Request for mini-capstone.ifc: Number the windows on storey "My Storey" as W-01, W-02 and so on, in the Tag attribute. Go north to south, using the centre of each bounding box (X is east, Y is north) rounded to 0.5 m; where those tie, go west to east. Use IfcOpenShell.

First a look at what the model holds.

```python
import ifcopenshell
import ifcopenshell.util.element
import ifcopenshell.util.placement

model = ifcopenshell.open("mini-capstone.ifc")
print(model.schema)
storey = next(s for s in model.by_type("IfcBuildingStorey") if s.Name == "My Storey")
windows = [e for e in ifcopenshell.util.element.get_decomposition(storey) if e.is_a("IfcWindow")]
for e in sorted(windows, key=lambda e: e.id()):
    origin = ifcopenshell.util.placement.get_local_placement(e.ObjectPlacement)[:3, 3]
    print(e.id(), e.Tag, e.Name, origin.round(2) + 0.0, sep=" | ")
```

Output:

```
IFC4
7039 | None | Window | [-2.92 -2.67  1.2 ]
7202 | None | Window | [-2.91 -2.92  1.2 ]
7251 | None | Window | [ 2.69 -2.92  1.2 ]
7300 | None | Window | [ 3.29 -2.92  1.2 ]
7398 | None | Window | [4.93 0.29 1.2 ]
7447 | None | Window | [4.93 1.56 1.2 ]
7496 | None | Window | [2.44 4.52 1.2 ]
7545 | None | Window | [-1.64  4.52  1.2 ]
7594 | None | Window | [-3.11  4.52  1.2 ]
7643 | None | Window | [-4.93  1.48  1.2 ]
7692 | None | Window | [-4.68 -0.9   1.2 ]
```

```python
import ifcopenshell
import ifcopenshell.geom
import ifcopenshell.util.element
import ifcopenshell.util.shape

model = ifcopenshell.open("mini-capstone.ifc")
settings = ifcopenshell.geom.settings()
settings.set("use-world-coords", True)


def centre(element):
    shape = ifcopenshell.geom.create_shape(settings, element)
    return ifcopenshell.util.shape.get_bbox_centroid(shape.geometry)


storey = next(s for s in model.by_type("IfcBuildingStorey") if s.Name == "My Storey")
windows = [e for e in ifcopenshell.util.element.get_decomposition(storey) if e.is_a("IfcWindow")]

# Insertion points can sit at a corner or the storey origin, so sort by the geometry (in metres).
centres = {e: centre(e) for e in windows}
windows.sort(key=lambda e: (-round(centres[e][1] / 0.5), centres[e][0]))

for i, e in enumerate(windows, start=1):
    number = f"W-{i:02d}"
    e.Tag = number
    print(e.id(), number)

model.write("mini-capstone_v2.ifc")
```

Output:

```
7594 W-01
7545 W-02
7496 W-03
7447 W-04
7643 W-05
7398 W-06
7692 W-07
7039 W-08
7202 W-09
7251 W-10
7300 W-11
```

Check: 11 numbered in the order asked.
